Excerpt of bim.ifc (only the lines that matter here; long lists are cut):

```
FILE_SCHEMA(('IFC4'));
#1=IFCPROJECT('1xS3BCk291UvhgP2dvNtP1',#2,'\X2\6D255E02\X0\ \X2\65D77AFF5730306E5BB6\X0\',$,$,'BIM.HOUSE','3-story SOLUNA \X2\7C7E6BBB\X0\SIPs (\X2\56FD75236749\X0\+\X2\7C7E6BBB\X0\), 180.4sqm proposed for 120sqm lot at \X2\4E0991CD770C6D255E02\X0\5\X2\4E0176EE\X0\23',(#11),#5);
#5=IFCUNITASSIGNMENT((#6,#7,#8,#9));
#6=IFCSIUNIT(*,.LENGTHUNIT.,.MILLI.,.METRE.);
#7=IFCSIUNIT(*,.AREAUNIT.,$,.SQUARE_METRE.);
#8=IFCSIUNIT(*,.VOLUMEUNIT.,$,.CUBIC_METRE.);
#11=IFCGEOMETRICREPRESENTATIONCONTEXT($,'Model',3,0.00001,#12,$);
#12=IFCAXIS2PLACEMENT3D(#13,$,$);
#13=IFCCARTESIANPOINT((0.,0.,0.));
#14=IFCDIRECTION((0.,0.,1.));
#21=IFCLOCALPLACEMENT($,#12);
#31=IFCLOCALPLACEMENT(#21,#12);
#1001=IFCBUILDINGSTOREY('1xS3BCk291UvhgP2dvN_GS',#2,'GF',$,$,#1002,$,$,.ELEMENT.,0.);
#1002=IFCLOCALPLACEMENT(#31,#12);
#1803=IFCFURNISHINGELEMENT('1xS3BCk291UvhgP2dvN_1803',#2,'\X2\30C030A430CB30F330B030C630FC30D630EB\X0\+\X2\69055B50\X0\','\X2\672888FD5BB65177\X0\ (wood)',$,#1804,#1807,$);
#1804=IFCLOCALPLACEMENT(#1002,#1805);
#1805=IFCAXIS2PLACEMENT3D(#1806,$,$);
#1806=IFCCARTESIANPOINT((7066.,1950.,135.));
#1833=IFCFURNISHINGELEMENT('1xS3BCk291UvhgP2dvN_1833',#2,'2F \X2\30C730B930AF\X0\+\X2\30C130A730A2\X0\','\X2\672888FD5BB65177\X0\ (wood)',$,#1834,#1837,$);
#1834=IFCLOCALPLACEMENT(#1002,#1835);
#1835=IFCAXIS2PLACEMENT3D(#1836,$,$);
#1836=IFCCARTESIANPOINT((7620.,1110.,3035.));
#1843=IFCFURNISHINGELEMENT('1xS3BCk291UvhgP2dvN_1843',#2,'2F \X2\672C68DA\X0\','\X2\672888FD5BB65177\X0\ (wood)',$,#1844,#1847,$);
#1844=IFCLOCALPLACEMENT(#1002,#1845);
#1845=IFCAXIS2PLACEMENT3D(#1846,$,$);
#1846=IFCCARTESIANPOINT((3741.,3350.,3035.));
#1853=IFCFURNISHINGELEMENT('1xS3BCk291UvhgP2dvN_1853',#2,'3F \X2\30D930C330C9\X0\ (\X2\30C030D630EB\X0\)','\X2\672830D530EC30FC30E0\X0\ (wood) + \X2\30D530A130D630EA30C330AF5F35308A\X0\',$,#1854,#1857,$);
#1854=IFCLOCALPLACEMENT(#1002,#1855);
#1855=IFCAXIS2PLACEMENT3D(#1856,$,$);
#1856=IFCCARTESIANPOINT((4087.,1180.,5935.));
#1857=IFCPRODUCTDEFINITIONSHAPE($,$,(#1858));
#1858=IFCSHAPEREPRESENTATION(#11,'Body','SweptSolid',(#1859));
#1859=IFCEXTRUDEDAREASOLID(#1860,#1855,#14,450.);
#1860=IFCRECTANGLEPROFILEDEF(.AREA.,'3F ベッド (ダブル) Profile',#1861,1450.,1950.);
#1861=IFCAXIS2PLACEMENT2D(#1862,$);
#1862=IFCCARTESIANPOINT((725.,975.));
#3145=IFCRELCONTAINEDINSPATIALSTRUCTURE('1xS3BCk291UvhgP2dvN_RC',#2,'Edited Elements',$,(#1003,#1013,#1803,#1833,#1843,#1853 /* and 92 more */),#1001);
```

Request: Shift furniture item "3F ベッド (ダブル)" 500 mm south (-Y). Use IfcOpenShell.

```python
import ifcopenshell
import ifcopenshell.api.geometry
import ifcopenshell.util.placement
import ifcopenshell.util.unit

model = ifcopenshell.open("bim.ifc")
unit_scale = ifcopenshell.util.unit.calculate_unit_scale(model)

item = model.by_guid("1xS3BCk291UvhgP2dvN_1853")
matrix = ifcopenshell.util.placement.get_local_placement(item.ObjectPlacement)
matrix[1, 3] -= 0.5 / unit_scale
ifcopenshell.api.geometry.edit_object_placement(model, product=item, matrix=matrix, is_si=False)

print(ifcopenshell.util.placement.get_local_placement(item.ObjectPlacement).round(3) + 0.0)

model.write("bim_rev.ifc")
```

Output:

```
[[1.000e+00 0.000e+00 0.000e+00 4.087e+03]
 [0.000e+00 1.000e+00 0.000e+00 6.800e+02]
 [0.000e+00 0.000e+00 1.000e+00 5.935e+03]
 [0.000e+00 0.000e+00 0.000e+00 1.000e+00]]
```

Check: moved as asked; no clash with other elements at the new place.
